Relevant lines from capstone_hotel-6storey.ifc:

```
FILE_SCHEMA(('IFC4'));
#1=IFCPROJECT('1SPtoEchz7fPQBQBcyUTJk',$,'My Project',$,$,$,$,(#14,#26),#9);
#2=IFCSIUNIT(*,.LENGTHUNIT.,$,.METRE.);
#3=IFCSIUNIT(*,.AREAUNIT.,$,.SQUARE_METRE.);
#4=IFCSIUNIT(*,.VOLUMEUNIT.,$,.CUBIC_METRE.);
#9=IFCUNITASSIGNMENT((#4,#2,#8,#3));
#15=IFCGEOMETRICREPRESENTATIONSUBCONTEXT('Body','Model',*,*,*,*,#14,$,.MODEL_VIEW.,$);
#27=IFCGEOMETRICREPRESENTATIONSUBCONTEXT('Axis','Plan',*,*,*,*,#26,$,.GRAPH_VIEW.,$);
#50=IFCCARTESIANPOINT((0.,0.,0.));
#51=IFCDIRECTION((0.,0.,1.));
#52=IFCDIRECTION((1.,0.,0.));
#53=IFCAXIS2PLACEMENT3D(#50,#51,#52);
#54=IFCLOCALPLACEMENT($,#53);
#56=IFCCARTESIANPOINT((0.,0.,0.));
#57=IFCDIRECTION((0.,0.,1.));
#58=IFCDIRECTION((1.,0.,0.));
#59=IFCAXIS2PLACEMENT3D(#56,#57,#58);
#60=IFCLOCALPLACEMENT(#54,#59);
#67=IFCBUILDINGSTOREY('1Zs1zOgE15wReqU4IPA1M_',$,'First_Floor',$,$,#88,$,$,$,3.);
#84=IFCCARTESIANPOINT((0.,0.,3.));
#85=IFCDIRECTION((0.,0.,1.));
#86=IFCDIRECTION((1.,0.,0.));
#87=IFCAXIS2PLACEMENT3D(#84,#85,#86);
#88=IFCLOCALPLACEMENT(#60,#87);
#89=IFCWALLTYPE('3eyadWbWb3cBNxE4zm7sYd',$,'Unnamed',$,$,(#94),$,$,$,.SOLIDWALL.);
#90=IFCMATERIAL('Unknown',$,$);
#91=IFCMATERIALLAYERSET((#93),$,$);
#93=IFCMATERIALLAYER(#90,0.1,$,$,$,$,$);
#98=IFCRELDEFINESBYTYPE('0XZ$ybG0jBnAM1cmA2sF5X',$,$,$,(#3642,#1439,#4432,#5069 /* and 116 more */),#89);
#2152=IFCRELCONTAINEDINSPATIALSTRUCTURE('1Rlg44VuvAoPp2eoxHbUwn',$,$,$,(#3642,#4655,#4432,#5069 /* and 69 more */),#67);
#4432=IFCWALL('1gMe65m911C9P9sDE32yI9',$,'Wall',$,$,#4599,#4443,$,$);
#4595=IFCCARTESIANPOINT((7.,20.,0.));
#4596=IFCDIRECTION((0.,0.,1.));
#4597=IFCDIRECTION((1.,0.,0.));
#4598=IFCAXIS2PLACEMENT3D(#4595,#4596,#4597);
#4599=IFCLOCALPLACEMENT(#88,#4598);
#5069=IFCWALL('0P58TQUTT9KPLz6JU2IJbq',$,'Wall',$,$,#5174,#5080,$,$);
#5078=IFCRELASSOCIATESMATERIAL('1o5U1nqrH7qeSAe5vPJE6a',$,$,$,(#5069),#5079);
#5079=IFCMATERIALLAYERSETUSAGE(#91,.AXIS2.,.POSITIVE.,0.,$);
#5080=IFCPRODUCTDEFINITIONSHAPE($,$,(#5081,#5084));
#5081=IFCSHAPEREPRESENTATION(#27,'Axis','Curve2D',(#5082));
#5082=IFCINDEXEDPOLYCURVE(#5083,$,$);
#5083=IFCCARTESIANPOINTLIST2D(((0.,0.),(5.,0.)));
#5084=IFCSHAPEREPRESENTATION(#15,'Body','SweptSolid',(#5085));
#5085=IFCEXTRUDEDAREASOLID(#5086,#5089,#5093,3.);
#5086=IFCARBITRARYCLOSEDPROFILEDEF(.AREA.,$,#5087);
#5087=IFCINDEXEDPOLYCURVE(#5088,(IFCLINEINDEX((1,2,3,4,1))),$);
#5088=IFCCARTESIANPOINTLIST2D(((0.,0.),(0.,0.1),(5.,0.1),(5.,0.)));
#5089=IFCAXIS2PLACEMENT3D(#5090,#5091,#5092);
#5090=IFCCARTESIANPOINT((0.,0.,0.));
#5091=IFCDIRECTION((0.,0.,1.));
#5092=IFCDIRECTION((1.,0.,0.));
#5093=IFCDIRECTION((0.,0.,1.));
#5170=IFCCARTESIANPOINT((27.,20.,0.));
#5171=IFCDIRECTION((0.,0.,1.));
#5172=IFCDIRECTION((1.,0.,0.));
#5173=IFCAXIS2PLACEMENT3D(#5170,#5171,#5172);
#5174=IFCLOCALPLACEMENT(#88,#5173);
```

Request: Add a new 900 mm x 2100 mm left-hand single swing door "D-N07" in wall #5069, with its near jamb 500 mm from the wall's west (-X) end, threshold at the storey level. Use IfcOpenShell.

```python
import numpy as np
import ifcopenshell
import ifcopenshell.api.feature
import ifcopenshell.api.geometry
import ifcopenshell.api.root
import ifcopenshell.api.spatial
import ifcopenshell.geom
import ifcopenshell.util.element
import ifcopenshell.util.placement
import ifcopenshell.util.representation
import ifcopenshell.util.shape
import ifcopenshell.util.unit

model = ifcopenshell.open("capstone_hotel-6storey.ifc")
unit_scale = ifcopenshell.util.unit.calculate_unit_scale(model)
settings = ifcopenshell.geom.settings()


def volume(element):
    """Net volume in cubic metres, openings subtracted."""
    shape = ifcopenshell.geom.create_shape(settings, element)
    return ifcopenshell.util.shape.get_volume(shape.geometry)


wall = model.by_guid("0P58TQUTT9KPLz6JU2IJbq")
storey = ifcopenshell.util.element.get_container(wall, ifc_class="IfcBuildingStorey")
context = ifcopenshell.util.representation.get_context(model, "Model", "Body", "MODEL_VIEW")
before = volume(wall)

width, height, from_end, sill = 0.9, 2.1, 0.5, 0.0  # metres

# The wall runs along its own X axis, and the end named is its -X end.
wall_shape = ifcopenshell.geom.create_shape(settings, wall)
x, y, z = ifcopenshell.util.shape.get_vertices(wall_shape.geometry).T
start = x.min() + from_end
face, thickness = float(y.min()), float(y.max() - y.min())
wall_matrix = ifcopenshell.util.placement.get_local_placement(wall.ObjectPlacement)
level = ifcopenshell.util.placement.get_local_placement(storey.ObjectPlacement)[2, 3]


def in_wall(x, y):
    """Placement at x, y metres in the wall's axes, at sill height."""
    matrix = wall_matrix.copy()
    matrix[:, 3] = wall_matrix @ np.array([x / unit_scale, y / unit_scale, 0.0, 1.0])
    matrix[2, 3] = level + sill / unit_scale
    return matrix


# Opening: a box that overshoots both wall faces by 50 mm.
opening = ifcopenshell.api.root.create_entity(model, ifc_class="IfcOpeningElement", predefined_type="OPENING")
box = ifcopenshell.api.geometry.add_wall_representation(
    model, context=context, length=width, height=height, thickness=thickness + 0.1
)
ifcopenshell.api.geometry.assign_representation(model, product=opening, representation=box)
ifcopenshell.api.geometry.edit_object_placement(model, product=opening, matrix=in_wall(start, face - 0.05), is_si=False)
ifcopenshell.api.feature.add_feature(model, feature=opening, element=wall)

door = ifcopenshell.api.root.create_entity(model, ifc_class="IfcDoor", name="D-N07", predefined_type="DOOR")
door.OverallWidth, door.OverallHeight = width / unit_scale, height / unit_scale
door.OperationType = "SINGLE_SWING_LEFT"
body = ifcopenshell.api.geometry.add_door_representation(
    model,
    context=context,
    overall_width=door.OverallWidth,
    overall_height=door.OverallHeight,
    operation_type="SINGLE_SWING_LEFT",
    lining_properties={"LiningDepth": thickness / unit_scale, "ThresholdDepth": thickness / unit_scale},
)
ifcopenshell.api.geometry.assign_representation(model, product=door, representation=body)
ifcopenshell.api.spatial.assign_container(model, products=[door], relating_structure=storey)
ifcopenshell.api.feature.add_filling(model, opening=opening, element=door)

# The lining spans the wall, so the door starts at the wall face.
ifcopenshell.api.geometry.edit_object_placement(model, product=door, matrix=in_wall(start, face), is_si=False)

after = volume(wall)

print(f"wall volume {before:.3f} -> {after:.3f} m3")

model.write("capstone_hotel-6storey_v2.ifc")
```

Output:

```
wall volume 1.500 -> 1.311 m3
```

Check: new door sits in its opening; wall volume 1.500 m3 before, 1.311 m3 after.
